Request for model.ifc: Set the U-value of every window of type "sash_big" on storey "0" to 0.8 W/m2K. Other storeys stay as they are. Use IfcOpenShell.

First a look at what the model holds.

```python
import ifcopenshell
import ifcopenshell.util.element

model = ifcopenshell.open("model.ifc")
print(model.schema)
storey = next(s for s in model.by_type("IfcBuildingStorey") if s.Name == "0")
windows = [e for e in ifcopenshell.util.element.get_decomposition(storey) if e.is_a("IfcWindow")]
seen = {}
for e in windows:
    element_type = ifcopenshell.util.element.get_type(e)
    key = (element_type.Name if element_type != e and element_type else None, ifcopenshell.util.element.get_pset(e, "Pset_WindowCommon", "ThermalTransmittance"))
    seen[key] = seen.get(key, 0) + 1
for (name, value), count in sorted(seen.items(), key=str):
    print(count, "x", name, "|", value)
```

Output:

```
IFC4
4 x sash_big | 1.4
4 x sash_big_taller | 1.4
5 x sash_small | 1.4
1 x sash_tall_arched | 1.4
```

```python
import ifcopenshell
import ifcopenshell.api.pset
import ifcopenshell.util.element

model = ifcopenshell.open("model.ifc")

storey = next(s for s in model.by_type("IfcBuildingStorey") if s.Name == "0")
windows = [e for e in ifcopenshell.util.element.get_decomposition(storey) if e.is_a("IfcWindow")]

count = 0
for e in windows:
    element_type = ifcopenshell.util.element.get_type(e)
    if element_type in (None, e) or element_type.Name != "sash_big":
        continue
    # add_pset returns the element's existing set when there is one.
    pset = ifcopenshell.api.pset.add_pset(model, product=e, name="Pset_WindowCommon")
    ifcopenshell.api.pset.edit_pset(model, pset=pset, properties={"ThermalTransmittance": 0.8})
    count += 1

print(count, "windows updated")

model.write("model_updated.ifc")
```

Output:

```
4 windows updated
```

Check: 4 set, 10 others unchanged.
